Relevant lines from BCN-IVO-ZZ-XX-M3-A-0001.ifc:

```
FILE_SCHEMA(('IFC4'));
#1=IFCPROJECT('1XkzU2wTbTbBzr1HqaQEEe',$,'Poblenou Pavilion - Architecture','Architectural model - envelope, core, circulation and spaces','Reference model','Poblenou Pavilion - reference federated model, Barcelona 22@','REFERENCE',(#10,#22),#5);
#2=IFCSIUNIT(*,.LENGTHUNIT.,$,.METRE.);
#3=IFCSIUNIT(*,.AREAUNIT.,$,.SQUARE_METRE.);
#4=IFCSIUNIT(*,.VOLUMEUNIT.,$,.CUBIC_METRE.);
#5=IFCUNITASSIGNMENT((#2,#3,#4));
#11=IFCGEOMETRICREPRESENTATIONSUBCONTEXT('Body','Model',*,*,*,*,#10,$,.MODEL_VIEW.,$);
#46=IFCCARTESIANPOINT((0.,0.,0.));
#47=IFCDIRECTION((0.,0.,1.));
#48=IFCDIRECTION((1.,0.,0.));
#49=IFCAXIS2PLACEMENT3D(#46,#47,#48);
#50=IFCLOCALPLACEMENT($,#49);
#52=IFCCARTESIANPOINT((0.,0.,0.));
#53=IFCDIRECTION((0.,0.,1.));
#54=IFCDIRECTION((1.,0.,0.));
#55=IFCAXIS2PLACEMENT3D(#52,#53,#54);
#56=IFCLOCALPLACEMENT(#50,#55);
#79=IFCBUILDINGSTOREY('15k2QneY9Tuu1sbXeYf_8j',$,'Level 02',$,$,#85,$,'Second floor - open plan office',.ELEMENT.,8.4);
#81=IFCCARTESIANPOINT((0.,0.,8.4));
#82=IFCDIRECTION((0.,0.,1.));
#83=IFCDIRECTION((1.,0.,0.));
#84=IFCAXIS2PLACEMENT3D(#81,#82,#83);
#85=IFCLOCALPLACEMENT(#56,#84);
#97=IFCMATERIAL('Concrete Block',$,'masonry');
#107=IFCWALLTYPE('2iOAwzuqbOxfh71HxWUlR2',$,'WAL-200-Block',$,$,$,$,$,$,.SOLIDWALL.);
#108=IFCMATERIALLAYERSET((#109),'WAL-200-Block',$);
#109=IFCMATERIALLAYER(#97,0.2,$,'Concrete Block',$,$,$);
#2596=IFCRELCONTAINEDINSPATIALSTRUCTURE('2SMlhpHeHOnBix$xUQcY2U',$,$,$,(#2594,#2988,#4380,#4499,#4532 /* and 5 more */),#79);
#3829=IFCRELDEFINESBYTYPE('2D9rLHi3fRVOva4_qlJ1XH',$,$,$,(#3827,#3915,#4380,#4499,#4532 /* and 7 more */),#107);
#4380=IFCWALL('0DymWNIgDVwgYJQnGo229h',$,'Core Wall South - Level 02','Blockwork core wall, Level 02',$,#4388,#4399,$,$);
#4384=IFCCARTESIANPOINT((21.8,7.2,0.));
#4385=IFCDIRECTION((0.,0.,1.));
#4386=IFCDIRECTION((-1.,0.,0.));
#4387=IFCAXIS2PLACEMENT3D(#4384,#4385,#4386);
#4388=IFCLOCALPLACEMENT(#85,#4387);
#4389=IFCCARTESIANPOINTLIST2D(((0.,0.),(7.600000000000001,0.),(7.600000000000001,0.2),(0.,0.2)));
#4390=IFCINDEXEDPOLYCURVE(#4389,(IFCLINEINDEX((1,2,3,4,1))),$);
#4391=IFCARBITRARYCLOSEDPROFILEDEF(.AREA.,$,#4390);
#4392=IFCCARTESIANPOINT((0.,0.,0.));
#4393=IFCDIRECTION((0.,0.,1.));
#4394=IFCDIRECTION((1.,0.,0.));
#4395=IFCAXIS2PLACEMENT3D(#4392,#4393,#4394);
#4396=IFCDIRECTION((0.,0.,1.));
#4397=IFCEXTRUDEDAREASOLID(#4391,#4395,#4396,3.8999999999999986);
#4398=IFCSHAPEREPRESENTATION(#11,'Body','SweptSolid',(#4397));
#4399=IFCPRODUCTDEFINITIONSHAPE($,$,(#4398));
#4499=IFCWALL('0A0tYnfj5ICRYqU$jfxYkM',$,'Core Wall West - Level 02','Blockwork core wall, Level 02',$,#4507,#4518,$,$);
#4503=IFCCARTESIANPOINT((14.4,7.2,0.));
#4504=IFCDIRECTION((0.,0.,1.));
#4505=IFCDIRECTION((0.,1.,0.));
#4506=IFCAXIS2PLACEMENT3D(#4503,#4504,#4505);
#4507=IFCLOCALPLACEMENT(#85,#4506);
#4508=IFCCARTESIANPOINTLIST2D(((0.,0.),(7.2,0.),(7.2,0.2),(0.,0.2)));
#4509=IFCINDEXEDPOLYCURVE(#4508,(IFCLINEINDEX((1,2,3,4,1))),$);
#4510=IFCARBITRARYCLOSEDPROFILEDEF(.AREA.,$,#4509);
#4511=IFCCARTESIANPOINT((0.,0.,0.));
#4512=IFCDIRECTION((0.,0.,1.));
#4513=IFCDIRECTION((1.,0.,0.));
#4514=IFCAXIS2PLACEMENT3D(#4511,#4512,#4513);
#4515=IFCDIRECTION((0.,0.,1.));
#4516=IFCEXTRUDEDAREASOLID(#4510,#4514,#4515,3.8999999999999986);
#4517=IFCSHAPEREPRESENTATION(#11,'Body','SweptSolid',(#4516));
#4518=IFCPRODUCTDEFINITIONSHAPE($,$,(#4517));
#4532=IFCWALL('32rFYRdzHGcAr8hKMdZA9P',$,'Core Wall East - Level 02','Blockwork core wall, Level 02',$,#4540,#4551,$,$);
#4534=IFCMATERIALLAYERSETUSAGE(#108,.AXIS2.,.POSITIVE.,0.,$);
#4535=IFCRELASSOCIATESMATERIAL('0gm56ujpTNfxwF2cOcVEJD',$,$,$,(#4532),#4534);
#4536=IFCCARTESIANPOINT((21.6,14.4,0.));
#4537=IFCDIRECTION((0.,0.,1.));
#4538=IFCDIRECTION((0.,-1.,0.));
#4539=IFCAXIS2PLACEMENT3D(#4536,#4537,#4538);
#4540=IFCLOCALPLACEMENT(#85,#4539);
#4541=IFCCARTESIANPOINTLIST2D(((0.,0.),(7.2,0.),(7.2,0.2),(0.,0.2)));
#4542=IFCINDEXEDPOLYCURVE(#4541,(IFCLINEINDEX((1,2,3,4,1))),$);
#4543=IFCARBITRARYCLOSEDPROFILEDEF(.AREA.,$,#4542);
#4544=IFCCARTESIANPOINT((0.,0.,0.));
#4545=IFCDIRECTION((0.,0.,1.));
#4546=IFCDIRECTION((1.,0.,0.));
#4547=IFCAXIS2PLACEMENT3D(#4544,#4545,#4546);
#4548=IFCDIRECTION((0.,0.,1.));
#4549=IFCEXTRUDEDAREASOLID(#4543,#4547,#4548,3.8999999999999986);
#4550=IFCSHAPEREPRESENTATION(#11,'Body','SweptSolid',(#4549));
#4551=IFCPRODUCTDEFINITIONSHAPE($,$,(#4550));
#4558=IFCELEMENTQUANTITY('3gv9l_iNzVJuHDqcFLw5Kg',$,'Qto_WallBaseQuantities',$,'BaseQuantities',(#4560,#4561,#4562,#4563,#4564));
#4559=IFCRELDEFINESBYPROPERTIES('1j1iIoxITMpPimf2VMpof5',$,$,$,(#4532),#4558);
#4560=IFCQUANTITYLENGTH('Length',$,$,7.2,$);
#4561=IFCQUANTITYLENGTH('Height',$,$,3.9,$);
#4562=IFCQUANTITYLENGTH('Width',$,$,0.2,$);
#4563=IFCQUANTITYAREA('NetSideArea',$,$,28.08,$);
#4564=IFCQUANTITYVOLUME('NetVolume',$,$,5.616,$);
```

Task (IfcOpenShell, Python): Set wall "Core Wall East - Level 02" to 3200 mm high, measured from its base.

```python
import ifcopenshell
import ifcopenshell.api.pset
import ifcopenshell.geom
import ifcopenshell.util.element
import ifcopenshell.util.representation
import ifcopenshell.util.shape
import ifcopenshell.util.unit

model = ifcopenshell.open("BCN-IVO-ZZ-XX-M3-A-0001.ifc")
unit_scale = ifcopenshell.util.unit.calculate_unit_scale(model)
area_scale = ifcopenshell.util.unit.calculate_unit_scale(model, "AREAUNIT")
volume_scale = ifcopenshell.util.unit.calculate_unit_scale(model, "VOLUMEUNIT")
settings = ifcopenshell.geom.settings()


def volume(element):
    """Net volume in cubic metres, openings subtracted."""
    shape = ifcopenshell.geom.create_shape(settings, element)
    return ifcopenshell.util.shape.get_volume(shape.geometry)


wall = model.by_id(4532)
before = volume(wall)

body = ifcopenshell.util.representation.get_representation(wall, "Model", "Body")
solid = body.Items[0]
old_height = solid.Depth
solid.Depth = 3.2 / unit_scale
after = volume(wall)
thickness = 0.2  # wall thickness in metres

# Update the stored height, areas and volumes.
qto = model.by_id(ifcopenshell.util.element.get_pset(wall, "Qto_WallBaseQuantities", should_inherit=False)["id"])
ifcopenshell.api.pset.edit_qto(model, qto=qto, properties={
    "Height": solid.Depth,
    "NetSideArea": after / thickness / area_scale,
    "NetVolume": after / volume_scale,
})

print(f"height {old_height:g} -> {solid.Depth:g}, volume {before:.3f} -> {after:.3f} m3")

model.write("BCN-IVO-ZZ-XX-M3-A-0001-out.ifc")
```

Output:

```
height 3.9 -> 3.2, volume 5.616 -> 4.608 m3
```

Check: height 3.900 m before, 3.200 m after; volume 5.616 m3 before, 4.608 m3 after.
